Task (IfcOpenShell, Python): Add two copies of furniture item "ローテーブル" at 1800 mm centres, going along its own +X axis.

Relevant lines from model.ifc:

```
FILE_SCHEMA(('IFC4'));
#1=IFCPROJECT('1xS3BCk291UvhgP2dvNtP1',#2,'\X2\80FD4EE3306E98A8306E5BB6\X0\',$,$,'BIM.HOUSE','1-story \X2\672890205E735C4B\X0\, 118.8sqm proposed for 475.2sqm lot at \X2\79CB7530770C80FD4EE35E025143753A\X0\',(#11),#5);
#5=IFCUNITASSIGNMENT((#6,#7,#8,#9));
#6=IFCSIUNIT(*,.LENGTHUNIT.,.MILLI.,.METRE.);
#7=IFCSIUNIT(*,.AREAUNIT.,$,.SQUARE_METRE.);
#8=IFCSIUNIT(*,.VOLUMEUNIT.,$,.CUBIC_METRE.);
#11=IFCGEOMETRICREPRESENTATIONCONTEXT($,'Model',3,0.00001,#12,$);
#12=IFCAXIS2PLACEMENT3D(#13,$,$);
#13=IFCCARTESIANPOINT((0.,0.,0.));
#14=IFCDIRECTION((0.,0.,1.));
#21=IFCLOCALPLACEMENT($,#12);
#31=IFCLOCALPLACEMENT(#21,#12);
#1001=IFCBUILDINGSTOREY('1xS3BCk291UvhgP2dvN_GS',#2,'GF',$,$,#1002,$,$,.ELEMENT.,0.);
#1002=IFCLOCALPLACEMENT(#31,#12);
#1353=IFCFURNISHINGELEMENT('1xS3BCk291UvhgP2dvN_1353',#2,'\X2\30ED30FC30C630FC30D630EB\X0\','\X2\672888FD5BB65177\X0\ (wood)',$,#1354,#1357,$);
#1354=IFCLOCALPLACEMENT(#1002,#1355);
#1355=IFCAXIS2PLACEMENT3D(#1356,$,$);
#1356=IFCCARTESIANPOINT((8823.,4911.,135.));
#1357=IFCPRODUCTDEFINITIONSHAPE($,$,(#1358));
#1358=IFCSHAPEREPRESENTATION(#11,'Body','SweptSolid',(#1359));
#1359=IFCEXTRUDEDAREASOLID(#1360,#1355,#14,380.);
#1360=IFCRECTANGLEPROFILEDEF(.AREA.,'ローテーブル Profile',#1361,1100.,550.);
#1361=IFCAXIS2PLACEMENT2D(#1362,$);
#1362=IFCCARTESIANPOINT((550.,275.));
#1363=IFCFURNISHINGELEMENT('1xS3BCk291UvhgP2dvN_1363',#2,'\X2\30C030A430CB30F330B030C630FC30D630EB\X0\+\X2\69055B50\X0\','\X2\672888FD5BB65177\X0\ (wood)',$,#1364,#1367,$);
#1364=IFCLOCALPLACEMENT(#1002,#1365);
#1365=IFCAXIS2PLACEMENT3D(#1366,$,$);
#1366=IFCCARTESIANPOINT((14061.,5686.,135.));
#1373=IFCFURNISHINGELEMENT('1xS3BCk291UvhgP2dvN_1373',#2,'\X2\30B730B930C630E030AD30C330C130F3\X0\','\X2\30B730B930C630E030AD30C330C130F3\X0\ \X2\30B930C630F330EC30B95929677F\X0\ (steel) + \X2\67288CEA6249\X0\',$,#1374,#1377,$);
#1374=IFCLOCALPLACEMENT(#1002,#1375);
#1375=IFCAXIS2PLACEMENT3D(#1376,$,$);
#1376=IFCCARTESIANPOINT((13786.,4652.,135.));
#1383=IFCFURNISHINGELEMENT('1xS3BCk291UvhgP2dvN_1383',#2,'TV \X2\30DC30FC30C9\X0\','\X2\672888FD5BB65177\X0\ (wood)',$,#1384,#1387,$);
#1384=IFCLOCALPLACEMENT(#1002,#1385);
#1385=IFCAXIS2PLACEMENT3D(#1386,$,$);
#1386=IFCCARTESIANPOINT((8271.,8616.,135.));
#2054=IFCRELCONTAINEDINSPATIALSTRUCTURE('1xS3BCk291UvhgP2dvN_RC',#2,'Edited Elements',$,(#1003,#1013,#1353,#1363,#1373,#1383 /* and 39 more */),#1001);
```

```python
import ifcopenshell
import ifcopenshell.api.geometry
import ifcopenshell.api.root
import ifcopenshell.util.element
import ifcopenshell.util.placement

model = ifcopenshell.open("model.ifc")


def reuse_history(source, copy):
    """copy_class also copies each property set's owner history, people and application; keep the originals."""
    for rel in copy.IsDefinedBy:
        if rel.is_a("IfcRelDefinesByProperties") and (history := rel.RelatingPropertyDefinition.OwnerHistory):
            rel.RelatingPropertyDefinition.OwnerHistory = source.OwnerHistory
            ifcopenshell.util.element.remove_deep2(model, history)


source = model.by_guid("1xS3BCk291UvhgP2dvN_1353")
base = ifcopenshell.util.placement.get_local_placement(source.ObjectPlacement)
step = base[:3, 0] * 1800.0

for i in range(1, 3):
    copy = ifcopenshell.api.root.copy_class(model, product=source)
    copy.Representation = ifcopenshell.util.element.copy_deep(
        model, source.Representation, exclude=["IfcGeometricRepresentationContext", "IfcRepresentationMap"]
    )
    reuse_history(source, copy)
    matrix = base.copy()
    matrix[:3, 3] += i * step
    print("added at", matrix[:3, 3].round(3) + 0.0)
    ifcopenshell.api.geometry.edit_object_placement(model, product=copy, matrix=matrix, is_si=False)

model.write("model_rev.ifc")
```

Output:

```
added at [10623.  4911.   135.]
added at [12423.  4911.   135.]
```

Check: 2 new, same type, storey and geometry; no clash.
